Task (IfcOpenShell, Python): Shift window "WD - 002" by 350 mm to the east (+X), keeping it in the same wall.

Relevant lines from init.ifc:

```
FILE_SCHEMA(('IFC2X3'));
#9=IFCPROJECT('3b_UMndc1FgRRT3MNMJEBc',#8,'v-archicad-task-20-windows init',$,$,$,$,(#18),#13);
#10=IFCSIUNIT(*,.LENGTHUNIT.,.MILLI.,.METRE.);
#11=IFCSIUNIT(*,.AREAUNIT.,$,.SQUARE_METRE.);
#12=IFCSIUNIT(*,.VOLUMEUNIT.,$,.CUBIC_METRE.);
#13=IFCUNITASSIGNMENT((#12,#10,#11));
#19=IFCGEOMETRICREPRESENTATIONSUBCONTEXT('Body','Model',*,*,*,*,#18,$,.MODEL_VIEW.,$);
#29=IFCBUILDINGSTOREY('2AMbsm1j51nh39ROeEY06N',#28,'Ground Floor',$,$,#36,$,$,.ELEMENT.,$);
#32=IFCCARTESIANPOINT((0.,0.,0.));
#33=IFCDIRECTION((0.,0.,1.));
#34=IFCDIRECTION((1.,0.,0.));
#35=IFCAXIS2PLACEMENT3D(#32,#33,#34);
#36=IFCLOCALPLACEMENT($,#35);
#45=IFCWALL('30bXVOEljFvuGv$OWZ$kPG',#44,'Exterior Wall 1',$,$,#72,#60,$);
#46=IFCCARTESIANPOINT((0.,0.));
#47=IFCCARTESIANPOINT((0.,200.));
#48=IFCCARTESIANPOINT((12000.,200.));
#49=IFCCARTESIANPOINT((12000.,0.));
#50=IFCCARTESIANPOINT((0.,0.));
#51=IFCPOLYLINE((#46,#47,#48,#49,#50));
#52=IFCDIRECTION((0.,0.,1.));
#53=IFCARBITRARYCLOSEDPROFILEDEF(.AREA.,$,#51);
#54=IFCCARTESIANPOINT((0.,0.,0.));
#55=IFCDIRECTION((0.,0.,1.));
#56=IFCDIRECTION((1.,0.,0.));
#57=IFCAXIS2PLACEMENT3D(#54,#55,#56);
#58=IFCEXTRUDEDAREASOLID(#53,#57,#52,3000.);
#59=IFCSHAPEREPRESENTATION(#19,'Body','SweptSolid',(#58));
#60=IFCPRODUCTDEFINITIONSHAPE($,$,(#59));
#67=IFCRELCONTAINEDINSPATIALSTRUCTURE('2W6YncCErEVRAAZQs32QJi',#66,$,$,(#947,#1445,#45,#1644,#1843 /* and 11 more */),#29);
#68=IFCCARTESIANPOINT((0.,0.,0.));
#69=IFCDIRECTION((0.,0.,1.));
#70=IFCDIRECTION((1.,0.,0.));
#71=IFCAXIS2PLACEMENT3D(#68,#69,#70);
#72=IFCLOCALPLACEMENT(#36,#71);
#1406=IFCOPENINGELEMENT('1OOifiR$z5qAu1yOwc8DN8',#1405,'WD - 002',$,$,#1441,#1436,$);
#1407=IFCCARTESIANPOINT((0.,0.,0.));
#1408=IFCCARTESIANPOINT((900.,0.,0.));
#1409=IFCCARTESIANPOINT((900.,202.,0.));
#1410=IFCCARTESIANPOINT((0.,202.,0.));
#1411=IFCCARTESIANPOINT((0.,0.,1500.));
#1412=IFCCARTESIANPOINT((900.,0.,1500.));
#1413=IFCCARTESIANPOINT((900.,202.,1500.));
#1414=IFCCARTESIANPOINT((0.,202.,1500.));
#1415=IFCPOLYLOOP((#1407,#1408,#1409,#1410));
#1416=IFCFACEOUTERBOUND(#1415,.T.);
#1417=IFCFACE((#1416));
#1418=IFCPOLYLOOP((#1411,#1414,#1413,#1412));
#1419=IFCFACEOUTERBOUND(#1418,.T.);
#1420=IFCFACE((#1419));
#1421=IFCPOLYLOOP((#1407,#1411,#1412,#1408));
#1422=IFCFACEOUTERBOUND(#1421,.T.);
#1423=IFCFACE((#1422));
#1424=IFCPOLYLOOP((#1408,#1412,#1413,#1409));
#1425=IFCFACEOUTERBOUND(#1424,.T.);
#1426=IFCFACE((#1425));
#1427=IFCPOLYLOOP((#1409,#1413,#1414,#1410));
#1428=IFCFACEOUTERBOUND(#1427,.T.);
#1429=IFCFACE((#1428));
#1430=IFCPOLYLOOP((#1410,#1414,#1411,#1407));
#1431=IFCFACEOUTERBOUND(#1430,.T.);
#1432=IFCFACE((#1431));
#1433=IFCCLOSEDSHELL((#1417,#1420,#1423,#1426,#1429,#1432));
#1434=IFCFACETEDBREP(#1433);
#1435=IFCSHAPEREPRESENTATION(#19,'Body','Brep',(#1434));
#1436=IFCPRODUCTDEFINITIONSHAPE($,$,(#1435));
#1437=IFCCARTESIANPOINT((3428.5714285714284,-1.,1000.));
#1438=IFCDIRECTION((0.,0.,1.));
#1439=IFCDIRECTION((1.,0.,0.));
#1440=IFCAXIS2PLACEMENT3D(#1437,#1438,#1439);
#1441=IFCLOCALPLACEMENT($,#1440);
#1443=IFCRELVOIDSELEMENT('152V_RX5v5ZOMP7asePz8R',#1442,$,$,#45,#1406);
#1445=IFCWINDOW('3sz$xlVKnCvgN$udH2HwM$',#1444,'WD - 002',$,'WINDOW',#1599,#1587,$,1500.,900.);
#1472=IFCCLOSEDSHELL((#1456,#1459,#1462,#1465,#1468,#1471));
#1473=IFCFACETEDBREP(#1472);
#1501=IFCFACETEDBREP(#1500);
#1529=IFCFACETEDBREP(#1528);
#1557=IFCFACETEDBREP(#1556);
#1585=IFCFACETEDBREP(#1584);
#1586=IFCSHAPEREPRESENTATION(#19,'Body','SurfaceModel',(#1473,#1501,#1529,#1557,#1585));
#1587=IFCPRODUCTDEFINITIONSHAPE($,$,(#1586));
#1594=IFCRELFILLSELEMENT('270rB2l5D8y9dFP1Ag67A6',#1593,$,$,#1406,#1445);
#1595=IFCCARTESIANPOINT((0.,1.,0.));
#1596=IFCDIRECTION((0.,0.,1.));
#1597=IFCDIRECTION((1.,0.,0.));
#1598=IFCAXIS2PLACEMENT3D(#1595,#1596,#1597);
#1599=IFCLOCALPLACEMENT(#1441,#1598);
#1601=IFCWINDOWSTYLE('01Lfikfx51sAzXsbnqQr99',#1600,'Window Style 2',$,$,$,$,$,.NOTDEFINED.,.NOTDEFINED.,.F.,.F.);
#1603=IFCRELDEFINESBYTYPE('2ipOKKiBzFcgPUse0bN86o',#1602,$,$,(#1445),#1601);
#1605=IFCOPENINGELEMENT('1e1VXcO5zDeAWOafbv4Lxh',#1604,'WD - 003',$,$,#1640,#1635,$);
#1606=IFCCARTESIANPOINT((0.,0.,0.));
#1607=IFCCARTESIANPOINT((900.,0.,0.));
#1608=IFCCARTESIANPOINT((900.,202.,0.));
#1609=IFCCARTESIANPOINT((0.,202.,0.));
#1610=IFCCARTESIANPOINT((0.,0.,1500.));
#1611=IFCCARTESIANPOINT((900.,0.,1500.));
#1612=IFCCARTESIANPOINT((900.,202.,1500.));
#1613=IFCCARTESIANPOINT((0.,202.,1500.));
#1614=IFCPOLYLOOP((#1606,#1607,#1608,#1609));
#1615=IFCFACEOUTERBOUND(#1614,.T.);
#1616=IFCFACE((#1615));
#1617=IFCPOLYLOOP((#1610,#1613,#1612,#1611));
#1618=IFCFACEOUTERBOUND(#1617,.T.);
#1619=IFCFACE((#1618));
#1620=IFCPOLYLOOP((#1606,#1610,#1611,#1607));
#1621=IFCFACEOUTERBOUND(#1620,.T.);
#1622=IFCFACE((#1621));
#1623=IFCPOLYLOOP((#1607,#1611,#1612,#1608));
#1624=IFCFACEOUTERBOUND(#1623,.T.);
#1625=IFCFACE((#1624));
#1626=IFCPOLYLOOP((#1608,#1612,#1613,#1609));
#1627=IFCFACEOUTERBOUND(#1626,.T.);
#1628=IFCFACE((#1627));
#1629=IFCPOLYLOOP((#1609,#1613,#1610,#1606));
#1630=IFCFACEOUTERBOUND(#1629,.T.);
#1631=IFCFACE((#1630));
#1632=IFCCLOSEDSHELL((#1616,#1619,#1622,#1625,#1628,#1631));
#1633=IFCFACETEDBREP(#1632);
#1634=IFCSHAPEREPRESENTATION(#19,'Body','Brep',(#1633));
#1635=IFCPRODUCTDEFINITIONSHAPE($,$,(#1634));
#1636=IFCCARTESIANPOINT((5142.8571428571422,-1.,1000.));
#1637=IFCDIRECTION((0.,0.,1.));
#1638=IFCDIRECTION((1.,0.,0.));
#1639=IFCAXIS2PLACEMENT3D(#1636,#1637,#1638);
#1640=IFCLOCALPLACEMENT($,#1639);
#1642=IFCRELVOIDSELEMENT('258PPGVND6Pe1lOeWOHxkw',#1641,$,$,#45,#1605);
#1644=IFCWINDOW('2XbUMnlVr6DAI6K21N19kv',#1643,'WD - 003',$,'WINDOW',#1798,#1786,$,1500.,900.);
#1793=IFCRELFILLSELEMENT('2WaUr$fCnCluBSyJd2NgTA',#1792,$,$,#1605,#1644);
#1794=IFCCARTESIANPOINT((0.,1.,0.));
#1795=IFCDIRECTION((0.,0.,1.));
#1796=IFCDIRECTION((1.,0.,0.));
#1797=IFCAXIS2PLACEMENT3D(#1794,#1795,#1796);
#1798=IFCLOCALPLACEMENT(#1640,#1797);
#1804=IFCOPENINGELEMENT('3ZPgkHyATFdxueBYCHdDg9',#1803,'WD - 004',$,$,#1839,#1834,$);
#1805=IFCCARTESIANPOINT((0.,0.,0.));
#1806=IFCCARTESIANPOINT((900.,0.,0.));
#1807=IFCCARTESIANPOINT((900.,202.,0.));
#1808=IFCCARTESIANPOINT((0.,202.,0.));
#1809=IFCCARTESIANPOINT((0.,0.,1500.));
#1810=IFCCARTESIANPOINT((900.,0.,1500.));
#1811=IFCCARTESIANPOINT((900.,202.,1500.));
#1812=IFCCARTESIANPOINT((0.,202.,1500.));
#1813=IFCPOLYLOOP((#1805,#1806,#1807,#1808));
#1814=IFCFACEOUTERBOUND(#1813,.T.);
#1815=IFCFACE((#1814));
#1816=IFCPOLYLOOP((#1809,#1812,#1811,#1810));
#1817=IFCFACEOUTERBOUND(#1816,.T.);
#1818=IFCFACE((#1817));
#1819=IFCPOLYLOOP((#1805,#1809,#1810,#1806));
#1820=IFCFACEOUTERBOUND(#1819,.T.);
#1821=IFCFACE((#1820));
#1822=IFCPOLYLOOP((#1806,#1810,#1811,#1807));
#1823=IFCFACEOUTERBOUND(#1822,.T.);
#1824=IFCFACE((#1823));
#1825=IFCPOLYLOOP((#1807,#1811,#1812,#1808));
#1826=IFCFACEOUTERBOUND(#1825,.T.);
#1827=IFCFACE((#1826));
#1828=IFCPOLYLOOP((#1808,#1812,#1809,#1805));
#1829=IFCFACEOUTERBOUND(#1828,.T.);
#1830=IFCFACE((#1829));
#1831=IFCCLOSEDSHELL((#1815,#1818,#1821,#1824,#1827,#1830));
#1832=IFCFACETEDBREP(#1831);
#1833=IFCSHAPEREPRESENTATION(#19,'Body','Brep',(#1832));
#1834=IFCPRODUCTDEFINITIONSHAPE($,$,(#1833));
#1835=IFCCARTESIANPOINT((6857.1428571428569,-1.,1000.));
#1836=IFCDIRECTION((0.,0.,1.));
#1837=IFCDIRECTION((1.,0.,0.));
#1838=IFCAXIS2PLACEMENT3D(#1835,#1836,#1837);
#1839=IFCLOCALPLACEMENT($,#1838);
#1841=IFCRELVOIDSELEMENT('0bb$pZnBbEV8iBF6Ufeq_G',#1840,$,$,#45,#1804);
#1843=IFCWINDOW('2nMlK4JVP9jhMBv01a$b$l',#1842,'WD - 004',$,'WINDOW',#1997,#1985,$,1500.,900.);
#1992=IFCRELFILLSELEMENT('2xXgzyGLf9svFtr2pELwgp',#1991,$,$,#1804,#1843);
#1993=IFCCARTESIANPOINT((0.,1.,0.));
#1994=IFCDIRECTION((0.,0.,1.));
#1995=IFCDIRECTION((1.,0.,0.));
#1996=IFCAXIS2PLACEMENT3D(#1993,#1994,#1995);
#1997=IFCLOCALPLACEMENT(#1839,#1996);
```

```python
import ifcopenshell
import ifcopenshell.api.geometry
import ifcopenshell.util.placement

model = ifcopenshell.open("init.ifc")

window = model.by_guid("3sz$xlVKnCvgN$udH2HwM$")
opening = window.FillsVoids[0].RelatingOpeningElement
wall = opening.VoidsElements[0].RelatingBuildingElement

wall_matrix = ifcopenshell.util.placement.get_local_placement(wall.ObjectPlacement)
shift = wall_matrix[:3, 0] * 350.0
before = ifcopenshell.util.placement.get_local_placement(window.ObjectPlacement)[:3, 3].copy()

# The window is placed relative to its opening, so it follows when the opening moves.
matrix = ifcopenshell.util.placement.get_local_placement(opening.ObjectPlacement)
matrix[:3, 3] += shift
ifcopenshell.api.geometry.edit_object_placement(
    model, product=opening, matrix=matrix, is_si=False, should_transform_children=True
)

after = ifcopenshell.util.placement.get_local_placement(window.ObjectPlacement)[:3, 3]
print("window moved by", (after - before).round(3) + 0.0)

model.write("init_updated.ifc")
```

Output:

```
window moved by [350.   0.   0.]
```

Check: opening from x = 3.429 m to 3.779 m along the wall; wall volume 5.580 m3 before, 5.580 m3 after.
